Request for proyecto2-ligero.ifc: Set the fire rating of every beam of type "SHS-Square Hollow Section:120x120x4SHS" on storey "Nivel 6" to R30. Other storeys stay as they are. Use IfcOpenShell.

First a look at what the model holds.

```python
import ifcopenshell
import ifcopenshell.util.element

model = ifcopenshell.open("proyecto2-ligero.ifc")
print(model.schema)
storey = next(s for s in model.by_type("IfcBuildingStorey") if s.Name == "Nivel 6")
beams = [e for e in ifcopenshell.util.element.get_decomposition(storey) if e.is_a("IfcBeam")]
seen = {}
for e in beams:
    element_type = ifcopenshell.util.element.get_type(e)
    key = (element_type.Name if element_type != e and element_type else None, ifcopenshell.util.element.get_pset(e, "Pset_BeamCommon", "FireRating"))
    seen[key] = seen.get(key, 0) + 1
for (name, value), count in sorted(seen.items(), key=str):
    print(count, "x", name, "|", value)
```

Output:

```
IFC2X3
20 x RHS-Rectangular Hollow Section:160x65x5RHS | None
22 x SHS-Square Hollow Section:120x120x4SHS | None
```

```python
import ifcopenshell
import ifcopenshell.api.pset
import ifcopenshell.util.element

model = ifcopenshell.open("proyecto2-ligero.ifc")

storey = next(s for s in model.by_type("IfcBuildingStorey") if s.Name == "Nivel 6")
beams = [e for e in ifcopenshell.util.element.get_decomposition(storey) if e.is_a("IfcBeam")]

count = 0
for e in beams:
    element_type = ifcopenshell.util.element.get_type(e)
    if element_type in (None, e) or element_type.Name != "SHS-Square Hollow Section:120x120x4SHS":
        continue
    # add_pset returns the element's existing set when there is one.
    pset = ifcopenshell.api.pset.add_pset(model, product=e, name="Pset_BeamCommon")
    ifcopenshell.api.pset.edit_pset(model, pset=pset, properties={"FireRating": "R30"})
    count += 1

print(count, "beams updated")

model.write("proyecto2-ligero_edited.ifc")
```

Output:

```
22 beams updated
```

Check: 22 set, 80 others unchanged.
